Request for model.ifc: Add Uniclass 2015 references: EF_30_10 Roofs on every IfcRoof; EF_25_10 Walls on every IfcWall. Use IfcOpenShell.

First a look at what the model holds.

```python
import ifcopenshell

model = ifcopenshell.open("model.ifc")
print(model.schema)
print("classifications:", [c.Name for c in model.by_type("IfcClassification")])
for ifc_class in ("IfcDoor", "IfcRoof", "IfcStair", "IfcWall", "IfcWindow"):
    print(ifc_class, len(model.by_type(ifc_class)))
```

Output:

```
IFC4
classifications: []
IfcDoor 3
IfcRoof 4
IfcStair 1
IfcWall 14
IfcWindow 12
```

```python
import ifcopenshell
import ifcopenshell.api.classification

model = ifcopenshell.open("model.ifc")

system = ifcopenshell.api.classification.add_classification(model, classification="Uniclass 2015")

codes = {
    "IfcRoof": ("EF_30_10", "Roofs"),
    "IfcWall": ("EF_25_10", "Walls"),
}
for ifc_class, (code, name) in codes.items():
    products = model.by_type(ifc_class)
    ifcopenshell.api.classification.add_reference(
        model, products=products, classification=system, identification=code, name=name
    )
    print(code, len(products))

model.write("model_updated.ifc")
```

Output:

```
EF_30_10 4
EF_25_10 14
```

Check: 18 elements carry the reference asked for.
